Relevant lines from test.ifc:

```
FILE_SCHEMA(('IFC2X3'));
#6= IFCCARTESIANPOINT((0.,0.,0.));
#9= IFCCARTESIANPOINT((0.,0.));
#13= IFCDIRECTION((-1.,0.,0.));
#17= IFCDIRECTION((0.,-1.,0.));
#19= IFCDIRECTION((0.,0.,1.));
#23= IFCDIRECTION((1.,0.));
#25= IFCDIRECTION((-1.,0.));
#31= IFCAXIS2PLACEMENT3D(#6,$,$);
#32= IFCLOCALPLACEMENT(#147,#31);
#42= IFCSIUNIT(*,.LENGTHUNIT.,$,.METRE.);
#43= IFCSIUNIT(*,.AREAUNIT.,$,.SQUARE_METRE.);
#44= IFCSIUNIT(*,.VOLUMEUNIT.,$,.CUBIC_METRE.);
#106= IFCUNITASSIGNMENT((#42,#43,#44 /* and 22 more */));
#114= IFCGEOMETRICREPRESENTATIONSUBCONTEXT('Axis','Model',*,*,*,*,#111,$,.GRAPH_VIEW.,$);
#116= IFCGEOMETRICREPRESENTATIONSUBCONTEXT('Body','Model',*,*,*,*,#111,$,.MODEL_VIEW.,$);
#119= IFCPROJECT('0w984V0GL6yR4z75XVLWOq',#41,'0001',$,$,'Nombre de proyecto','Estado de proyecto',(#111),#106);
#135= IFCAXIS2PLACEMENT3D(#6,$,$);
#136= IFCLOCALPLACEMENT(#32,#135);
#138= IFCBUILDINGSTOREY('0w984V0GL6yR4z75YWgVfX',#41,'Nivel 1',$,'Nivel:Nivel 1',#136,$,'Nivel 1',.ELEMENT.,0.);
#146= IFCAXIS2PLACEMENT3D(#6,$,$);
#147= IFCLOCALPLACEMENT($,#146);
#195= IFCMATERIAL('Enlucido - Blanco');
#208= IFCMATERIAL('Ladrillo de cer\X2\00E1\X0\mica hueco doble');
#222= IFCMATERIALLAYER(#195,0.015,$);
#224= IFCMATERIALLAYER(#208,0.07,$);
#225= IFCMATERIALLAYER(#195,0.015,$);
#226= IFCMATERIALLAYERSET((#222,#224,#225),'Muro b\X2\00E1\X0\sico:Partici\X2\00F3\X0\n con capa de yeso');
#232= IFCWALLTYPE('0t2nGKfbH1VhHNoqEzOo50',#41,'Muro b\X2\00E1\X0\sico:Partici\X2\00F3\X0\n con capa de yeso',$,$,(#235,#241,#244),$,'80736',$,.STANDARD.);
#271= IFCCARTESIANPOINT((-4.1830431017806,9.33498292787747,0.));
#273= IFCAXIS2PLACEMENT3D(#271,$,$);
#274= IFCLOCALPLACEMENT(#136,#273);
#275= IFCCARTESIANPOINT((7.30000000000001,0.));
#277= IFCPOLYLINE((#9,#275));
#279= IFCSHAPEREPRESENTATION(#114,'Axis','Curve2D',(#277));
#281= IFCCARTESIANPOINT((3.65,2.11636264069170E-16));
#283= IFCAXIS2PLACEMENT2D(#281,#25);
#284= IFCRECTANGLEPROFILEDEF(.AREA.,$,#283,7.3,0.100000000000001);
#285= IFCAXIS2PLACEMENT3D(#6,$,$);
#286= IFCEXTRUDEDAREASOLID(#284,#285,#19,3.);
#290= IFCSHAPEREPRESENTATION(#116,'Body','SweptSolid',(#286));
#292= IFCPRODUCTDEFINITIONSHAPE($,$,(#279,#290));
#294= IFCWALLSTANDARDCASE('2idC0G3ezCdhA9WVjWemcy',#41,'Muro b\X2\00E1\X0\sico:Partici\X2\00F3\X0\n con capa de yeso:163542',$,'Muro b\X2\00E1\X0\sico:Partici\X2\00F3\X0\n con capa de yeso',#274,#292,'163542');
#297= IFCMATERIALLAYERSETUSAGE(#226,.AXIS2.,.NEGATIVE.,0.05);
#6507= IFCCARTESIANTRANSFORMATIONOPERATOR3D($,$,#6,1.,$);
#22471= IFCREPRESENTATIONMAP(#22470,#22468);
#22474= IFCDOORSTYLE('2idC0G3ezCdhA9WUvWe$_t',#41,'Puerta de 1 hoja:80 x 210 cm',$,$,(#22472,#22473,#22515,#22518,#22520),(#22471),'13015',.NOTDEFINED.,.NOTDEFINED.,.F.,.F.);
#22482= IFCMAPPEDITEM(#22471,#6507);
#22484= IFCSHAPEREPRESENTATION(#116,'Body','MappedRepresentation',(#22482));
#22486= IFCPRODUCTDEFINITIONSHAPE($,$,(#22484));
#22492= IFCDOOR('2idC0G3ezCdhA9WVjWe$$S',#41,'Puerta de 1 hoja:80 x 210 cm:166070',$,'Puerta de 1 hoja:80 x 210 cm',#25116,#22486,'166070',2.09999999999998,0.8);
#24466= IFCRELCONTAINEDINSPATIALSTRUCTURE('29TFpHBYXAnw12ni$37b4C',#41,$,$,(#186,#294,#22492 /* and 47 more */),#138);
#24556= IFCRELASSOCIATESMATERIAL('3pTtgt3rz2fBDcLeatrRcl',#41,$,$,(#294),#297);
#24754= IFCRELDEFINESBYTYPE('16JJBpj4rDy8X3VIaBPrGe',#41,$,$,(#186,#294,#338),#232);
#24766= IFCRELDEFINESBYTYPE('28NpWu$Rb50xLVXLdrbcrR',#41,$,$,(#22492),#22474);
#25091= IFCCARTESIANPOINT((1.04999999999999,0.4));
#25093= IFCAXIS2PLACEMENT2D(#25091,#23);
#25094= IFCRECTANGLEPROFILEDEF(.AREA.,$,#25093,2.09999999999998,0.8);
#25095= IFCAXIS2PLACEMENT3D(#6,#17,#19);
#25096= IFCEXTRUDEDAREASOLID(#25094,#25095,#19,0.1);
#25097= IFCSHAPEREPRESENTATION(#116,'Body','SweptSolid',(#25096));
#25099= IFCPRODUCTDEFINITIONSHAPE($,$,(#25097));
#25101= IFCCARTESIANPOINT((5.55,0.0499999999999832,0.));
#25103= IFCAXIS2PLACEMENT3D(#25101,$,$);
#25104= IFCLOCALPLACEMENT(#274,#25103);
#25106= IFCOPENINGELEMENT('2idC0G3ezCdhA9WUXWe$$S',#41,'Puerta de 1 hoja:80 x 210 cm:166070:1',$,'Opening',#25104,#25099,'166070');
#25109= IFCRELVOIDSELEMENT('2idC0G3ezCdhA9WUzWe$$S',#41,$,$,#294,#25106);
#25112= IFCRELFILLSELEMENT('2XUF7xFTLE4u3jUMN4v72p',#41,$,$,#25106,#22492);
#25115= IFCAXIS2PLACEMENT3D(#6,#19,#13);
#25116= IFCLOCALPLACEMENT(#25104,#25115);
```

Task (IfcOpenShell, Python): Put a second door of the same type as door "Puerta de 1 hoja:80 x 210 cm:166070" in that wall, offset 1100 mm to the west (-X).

```python
import ifcopenshell
import ifcopenshell.api.feature
import ifcopenshell.api.geometry
import ifcopenshell.api.root
import ifcopenshell.geom
import ifcopenshell.util.element
import ifcopenshell.util.placement
import ifcopenshell.util.shape
import ifcopenshell.util.unit

model = ifcopenshell.open("test.ifc")
unit_scale = ifcopenshell.util.unit.calculate_unit_scale(model)
settings = ifcopenshell.geom.settings()


def volume(element):
    """Net volume in cubic metres, openings subtracted."""
    shape = ifcopenshell.geom.create_shape(settings, element)
    return ifcopenshell.util.shape.get_volume(shape.geometry)


def reuse_history(source, copy):
    """copy_class also copies each property set's owner history, people and application; keep the originals."""
    for rel in copy.IsDefinedBy:
        if rel.is_a("IfcRelDefinesByProperties") and (history := rel.RelatingPropertyDefinition.OwnerHistory):
            rel.RelatingPropertyDefinition.OwnerHistory = source.OwnerHistory
            ifcopenshell.util.element.remove_deep2(model, history)


door = model.by_guid("2idC0G3ezCdhA9WVjWe$$S")
opening = door.FillsVoids[0].RelatingOpeningElement
wall = opening.VoidsElements[0].RelatingBuildingElement
before = volume(wall)
shift = ifcopenshell.util.placement.get_local_placement(wall.ObjectPlacement)[:3, 0] * -1.1 / unit_scale

# copy_class copies the void relationship, type, container and properties, but no geometry.
new_opening = ifcopenshell.api.root.copy_class(model, product=opening)
new_opening.Representation = ifcopenshell.util.element.copy_deep(
    model, opening.Representation, exclude=["IfcGeometricRepresentationContext", "IfcRepresentationMap"]
)
new_opening.Name = "Puerta de 1 hoja:80 x 210 cm"
new_opening.Tag = None
new_door = ifcopenshell.api.root.copy_class(model, product=door)
new_door.Representation = ifcopenshell.util.element.copy_deep(
    model, door.Representation, exclude=["IfcGeometricRepresentationContext", "IfcRepresentationMap"]
)
new_door.Name = "Puerta de 1 hoja:80 x 210 cm"
new_door.Tag = None
reuse_history(door, new_door)
fills = ifcopenshell.api.feature.add_filling(model, opening=new_opening, element=new_door)
fills.OwnerHistory = new_door.OwnerHistory  # required in IFC2X3

for old, new in ((opening, new_opening), (door, new_door)):
    matrix = ifcopenshell.util.placement.get_local_placement(old.ObjectPlacement)
    matrix[:3, 3] += shift
    ifcopenshell.api.geometry.edit_object_placement(model, product=new, matrix=matrix, is_si=False)

after = volume(wall)

print(f"wall volume {before:.3f} -> {after:.3f} m3")

model.write("test-out.ifc")
```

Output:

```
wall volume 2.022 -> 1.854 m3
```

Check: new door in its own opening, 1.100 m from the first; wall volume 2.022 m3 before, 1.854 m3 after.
